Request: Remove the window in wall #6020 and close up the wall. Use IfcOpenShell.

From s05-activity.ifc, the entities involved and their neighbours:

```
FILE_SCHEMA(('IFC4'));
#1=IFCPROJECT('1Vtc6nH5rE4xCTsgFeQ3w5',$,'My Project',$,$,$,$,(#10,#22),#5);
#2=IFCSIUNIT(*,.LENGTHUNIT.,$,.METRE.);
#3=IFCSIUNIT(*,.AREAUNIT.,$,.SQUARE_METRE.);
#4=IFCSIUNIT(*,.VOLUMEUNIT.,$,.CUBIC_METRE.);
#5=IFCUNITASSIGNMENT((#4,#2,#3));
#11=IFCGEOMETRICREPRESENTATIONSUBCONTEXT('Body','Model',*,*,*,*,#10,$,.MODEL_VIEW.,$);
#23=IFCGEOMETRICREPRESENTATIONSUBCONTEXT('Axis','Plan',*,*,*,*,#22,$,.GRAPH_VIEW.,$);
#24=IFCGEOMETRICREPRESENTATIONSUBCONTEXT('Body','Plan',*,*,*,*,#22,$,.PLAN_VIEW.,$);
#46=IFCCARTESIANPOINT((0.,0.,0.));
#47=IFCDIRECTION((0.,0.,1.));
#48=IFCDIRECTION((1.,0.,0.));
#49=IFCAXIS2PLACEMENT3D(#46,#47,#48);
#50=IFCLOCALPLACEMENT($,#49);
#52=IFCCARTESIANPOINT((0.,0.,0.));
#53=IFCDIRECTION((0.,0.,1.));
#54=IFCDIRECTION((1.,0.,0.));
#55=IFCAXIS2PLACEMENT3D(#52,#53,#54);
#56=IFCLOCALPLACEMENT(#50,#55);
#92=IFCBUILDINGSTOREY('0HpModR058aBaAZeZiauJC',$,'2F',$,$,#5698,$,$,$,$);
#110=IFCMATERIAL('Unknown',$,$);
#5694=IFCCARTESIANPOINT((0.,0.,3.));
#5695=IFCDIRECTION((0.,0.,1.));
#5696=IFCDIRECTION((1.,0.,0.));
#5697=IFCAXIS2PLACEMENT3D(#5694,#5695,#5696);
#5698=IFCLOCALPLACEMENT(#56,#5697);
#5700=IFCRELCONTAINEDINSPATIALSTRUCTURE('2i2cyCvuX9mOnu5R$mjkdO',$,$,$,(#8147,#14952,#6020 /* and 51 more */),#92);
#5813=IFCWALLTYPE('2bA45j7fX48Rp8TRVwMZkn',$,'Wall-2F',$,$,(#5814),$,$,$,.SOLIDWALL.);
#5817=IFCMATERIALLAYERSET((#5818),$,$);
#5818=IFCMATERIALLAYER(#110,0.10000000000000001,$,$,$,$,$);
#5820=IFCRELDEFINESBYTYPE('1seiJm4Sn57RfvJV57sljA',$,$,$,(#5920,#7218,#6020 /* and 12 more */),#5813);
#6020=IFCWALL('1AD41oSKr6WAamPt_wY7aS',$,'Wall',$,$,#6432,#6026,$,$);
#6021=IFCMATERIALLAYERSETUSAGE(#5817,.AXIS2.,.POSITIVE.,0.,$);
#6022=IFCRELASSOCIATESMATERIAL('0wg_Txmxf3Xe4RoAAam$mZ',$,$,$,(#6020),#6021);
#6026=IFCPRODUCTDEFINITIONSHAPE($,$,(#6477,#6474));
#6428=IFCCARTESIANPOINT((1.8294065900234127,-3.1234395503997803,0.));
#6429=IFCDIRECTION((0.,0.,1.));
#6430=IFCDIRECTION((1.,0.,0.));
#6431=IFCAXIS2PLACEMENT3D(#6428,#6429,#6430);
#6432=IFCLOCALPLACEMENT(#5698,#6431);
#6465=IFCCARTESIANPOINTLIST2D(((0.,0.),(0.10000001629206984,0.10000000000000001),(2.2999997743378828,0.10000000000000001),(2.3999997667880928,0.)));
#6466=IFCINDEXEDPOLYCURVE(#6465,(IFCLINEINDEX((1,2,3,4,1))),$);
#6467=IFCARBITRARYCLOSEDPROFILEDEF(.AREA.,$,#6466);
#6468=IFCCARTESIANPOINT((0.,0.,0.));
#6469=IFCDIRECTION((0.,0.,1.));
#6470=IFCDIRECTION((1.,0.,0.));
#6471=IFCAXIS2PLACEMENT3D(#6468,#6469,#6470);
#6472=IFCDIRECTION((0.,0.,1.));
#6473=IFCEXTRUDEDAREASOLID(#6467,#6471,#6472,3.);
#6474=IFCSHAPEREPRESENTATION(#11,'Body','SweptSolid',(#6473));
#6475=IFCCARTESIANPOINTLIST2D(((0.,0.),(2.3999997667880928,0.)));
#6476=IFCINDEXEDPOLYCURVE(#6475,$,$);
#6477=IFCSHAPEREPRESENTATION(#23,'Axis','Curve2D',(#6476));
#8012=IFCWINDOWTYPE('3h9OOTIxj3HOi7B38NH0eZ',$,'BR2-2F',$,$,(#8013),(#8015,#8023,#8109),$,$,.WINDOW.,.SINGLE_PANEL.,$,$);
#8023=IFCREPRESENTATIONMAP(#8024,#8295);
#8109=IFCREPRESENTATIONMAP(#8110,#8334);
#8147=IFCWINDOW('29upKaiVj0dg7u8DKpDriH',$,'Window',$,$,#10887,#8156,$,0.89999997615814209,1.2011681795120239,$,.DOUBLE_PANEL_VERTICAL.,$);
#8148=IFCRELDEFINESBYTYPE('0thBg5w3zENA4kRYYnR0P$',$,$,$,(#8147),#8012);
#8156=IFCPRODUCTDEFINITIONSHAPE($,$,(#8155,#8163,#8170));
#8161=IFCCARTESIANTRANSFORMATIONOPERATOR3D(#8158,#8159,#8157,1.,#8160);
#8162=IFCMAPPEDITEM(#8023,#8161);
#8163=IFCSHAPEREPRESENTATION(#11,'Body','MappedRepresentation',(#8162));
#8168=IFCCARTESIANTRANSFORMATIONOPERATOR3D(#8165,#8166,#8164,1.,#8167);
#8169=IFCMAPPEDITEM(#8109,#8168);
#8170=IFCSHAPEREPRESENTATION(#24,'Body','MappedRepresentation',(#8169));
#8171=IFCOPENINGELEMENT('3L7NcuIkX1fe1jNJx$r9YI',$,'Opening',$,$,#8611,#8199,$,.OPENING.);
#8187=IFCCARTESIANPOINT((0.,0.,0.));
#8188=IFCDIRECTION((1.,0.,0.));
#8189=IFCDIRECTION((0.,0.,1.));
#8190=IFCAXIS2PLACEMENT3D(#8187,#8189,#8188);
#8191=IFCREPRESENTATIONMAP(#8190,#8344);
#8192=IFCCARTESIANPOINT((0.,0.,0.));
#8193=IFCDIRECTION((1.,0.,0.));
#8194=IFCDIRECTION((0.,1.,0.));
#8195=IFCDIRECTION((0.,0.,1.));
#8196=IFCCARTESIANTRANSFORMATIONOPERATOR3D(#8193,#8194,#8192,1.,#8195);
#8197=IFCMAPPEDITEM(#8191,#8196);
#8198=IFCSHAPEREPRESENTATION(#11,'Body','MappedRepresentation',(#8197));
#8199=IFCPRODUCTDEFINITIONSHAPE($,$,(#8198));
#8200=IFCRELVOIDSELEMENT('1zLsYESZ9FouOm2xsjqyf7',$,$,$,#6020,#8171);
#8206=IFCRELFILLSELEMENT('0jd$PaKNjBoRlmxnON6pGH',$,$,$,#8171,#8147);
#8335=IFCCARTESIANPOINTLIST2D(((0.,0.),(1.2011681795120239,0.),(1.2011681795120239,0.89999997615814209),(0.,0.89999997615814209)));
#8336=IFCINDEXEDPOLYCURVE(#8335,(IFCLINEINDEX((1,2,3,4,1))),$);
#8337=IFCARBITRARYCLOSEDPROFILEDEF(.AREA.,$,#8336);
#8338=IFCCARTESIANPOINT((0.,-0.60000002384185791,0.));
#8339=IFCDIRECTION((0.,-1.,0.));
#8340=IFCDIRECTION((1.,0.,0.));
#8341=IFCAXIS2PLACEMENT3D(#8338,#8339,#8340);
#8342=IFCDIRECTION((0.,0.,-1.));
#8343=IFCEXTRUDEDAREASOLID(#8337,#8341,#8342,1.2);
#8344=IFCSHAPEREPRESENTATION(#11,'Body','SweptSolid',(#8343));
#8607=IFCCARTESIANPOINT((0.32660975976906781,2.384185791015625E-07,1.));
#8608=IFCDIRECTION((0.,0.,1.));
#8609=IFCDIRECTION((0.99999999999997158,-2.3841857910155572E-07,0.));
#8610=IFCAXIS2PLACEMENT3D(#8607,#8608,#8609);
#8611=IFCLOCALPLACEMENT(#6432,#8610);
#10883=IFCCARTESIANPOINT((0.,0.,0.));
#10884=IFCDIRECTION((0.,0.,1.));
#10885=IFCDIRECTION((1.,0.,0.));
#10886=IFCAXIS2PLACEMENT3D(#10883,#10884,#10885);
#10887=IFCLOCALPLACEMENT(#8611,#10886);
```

```python
import ifcopenshell
import ifcopenshell.api.feature
import ifcopenshell.api.root
import ifcopenshell.geom
import ifcopenshell.util.shape

model = ifcopenshell.open("s05-activity.ifc")
settings = ifcopenshell.geom.settings()


def volume(element):
    """Net volume in cubic metres, openings subtracted."""
    shape = ifcopenshell.geom.create_shape(settings, element)
    return ifcopenshell.util.shape.get_volume(shape.geometry)


window = model.by_guid("29upKaiVj0dg7u8DKpDriH")
opening = window.FillsVoids[0].RelatingOpeningElement
wall = opening.VoidsElements[0].RelatingBuildingElement
before = volume(wall)

ifcopenshell.api.root.remove_product(model, product=window)
ifcopenshell.api.feature.remove_feature(model, feature=opening)

after = volume(wall)

print(f"wall volume {before:.3f} -> {after:.3f} m3")

model.write("s05-activity_v2.ifc")
```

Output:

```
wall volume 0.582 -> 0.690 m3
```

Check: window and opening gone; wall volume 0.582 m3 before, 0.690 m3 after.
